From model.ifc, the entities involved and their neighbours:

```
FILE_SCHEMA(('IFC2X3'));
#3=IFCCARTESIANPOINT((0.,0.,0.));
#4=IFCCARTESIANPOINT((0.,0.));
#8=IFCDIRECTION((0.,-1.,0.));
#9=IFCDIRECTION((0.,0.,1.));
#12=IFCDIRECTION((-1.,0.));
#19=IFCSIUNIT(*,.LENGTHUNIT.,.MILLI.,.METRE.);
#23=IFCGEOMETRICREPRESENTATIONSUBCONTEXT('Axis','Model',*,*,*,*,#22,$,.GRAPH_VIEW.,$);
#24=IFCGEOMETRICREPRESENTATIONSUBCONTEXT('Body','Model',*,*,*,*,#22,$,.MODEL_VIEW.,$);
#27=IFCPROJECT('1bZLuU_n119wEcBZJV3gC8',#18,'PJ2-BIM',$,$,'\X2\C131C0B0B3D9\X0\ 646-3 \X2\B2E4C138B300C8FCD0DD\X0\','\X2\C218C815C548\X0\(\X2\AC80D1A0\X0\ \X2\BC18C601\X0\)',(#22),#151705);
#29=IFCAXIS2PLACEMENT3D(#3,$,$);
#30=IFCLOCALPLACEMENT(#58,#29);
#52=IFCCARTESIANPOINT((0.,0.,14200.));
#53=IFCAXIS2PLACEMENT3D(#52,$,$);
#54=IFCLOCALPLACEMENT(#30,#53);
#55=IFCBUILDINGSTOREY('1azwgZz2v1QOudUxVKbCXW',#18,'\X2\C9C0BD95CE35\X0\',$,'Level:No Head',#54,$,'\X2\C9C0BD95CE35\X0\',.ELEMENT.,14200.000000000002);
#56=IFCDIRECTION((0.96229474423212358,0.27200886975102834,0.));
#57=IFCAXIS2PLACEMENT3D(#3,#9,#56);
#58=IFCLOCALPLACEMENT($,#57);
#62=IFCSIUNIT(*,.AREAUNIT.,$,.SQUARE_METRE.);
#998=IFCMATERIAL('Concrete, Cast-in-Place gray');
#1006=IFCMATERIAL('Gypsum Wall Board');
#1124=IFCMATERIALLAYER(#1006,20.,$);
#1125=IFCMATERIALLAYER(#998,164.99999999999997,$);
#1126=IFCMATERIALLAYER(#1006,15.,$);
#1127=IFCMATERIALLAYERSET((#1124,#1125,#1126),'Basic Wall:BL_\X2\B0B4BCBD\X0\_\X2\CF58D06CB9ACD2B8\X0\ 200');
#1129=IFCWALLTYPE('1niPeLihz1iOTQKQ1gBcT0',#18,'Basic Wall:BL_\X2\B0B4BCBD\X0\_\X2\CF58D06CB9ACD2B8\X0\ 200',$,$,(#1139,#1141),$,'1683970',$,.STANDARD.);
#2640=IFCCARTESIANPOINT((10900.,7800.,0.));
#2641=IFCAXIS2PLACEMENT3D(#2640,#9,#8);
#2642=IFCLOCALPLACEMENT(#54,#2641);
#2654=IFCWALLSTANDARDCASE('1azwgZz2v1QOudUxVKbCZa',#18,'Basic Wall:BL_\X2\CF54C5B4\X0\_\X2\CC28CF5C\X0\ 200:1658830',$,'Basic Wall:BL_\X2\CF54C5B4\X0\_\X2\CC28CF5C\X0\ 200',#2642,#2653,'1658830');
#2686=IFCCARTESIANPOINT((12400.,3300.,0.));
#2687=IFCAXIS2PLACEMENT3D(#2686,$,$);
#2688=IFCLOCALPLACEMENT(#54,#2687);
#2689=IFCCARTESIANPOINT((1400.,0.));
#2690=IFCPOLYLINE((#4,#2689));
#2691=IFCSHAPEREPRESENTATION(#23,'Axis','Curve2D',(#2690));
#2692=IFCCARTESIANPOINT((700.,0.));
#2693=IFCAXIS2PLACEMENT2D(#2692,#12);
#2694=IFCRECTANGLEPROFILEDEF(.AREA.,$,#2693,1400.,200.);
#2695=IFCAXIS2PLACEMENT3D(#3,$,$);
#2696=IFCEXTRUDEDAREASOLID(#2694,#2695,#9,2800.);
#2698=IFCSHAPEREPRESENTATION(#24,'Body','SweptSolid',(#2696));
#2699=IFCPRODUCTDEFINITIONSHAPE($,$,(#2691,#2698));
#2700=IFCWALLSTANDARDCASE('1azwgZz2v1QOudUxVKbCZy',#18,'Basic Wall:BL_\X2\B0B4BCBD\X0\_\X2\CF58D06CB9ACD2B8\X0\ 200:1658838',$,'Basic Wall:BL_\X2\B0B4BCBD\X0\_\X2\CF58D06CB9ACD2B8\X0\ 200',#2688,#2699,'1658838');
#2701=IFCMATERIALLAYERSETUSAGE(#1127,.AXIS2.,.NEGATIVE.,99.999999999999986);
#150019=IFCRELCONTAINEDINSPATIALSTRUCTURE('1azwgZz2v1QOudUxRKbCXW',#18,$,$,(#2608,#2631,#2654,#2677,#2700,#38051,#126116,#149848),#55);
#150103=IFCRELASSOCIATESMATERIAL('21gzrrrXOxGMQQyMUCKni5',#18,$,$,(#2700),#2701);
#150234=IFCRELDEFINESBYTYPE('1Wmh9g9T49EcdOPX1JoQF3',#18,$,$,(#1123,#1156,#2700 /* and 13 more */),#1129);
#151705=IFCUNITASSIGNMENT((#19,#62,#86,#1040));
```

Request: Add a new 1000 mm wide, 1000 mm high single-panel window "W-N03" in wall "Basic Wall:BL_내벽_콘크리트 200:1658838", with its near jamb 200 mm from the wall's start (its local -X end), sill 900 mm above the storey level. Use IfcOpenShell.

```python
import numpy as np
import ifcopenshell
import ifcopenshell.api.feature
import ifcopenshell.api.geometry
import ifcopenshell.api.root
import ifcopenshell.api.spatial
import ifcopenshell.api.type
import ifcopenshell.geom
import ifcopenshell.util.element
import ifcopenshell.util.placement
import ifcopenshell.util.representation
import ifcopenshell.util.shape
import ifcopenshell.util.unit

model = ifcopenshell.open("model.ifc")
unit_scale = ifcopenshell.util.unit.calculate_unit_scale(model)
settings = ifcopenshell.geom.settings()


def volume(element):
    """Net volume in cubic metres, openings subtracted."""
    shape = ifcopenshell.geom.create_shape(settings, element)
    return ifcopenshell.util.shape.get_volume(shape.geometry)


wall = model.by_guid("1azwgZz2v1QOudUxVKbCZy")
storey = ifcopenshell.util.element.get_container(wall, ifc_class="IfcBuildingStorey")
context = ifcopenshell.util.representation.get_context(model, "Model", "Body", "MODEL_VIEW")
before = volume(wall)

width, height, from_end, sill = 1, 1, 0.2, 0.9  # metres

# The wall runs along its own X axis, and the end named is its -X end.
wall_shape = ifcopenshell.geom.create_shape(settings, wall)
x, y, z = ifcopenshell.util.shape.get_vertices(wall_shape.geometry).T
start = x.min() + from_end
face, thickness = float(y.min()), float(y.max() - y.min())
wall_matrix = ifcopenshell.util.placement.get_local_placement(wall.ObjectPlacement)
level = ifcopenshell.util.placement.get_local_placement(storey.ObjectPlacement)[2, 3]


def in_wall(x, y):
    """Placement at x, y metres in the wall's axes, at sill height."""
    matrix = wall_matrix.copy()
    matrix[:, 3] = wall_matrix @ np.array([x / unit_scale, y / unit_scale, 0.0, 1.0])
    matrix[2, 3] = level + sill / unit_scale
    return matrix


# Opening: a box that overshoots both wall faces by 50 mm.
opening = ifcopenshell.api.root.create_entity(model, ifc_class="IfcOpeningElement")
box = ifcopenshell.api.geometry.add_wall_representation(
    model, context=context, length=width, height=height, thickness=thickness + 0.1
)
ifcopenshell.api.geometry.assign_representation(model, product=opening, representation=box)
ifcopenshell.api.geometry.edit_object_placement(model, product=opening, matrix=in_wall(start, face - 0.05), is_si=False)
ifcopenshell.api.feature.add_feature(model, feature=opening, element=wall)

window = ifcopenshell.api.root.create_entity(model, ifc_class="IfcWindow", name="W-N03")
window.OverallWidth, window.OverallHeight = width / unit_scale, height / unit_scale
body = ifcopenshell.api.geometry.add_window_representation(
    model,
    context=context,
    overall_width=window.OverallWidth,
    overall_height=window.OverallHeight,
    partition_type="SINGLE_PANEL",
)
ifcopenshell.api.geometry.assign_representation(model, product=window, representation=body)
ifcopenshell.api.spatial.assign_container(model, products=[window], relating_structure=storey)
fills = ifcopenshell.api.feature.add_filling(model, opening=opening, element=window)
fills.OwnerHistory = window.OwnerHistory  # required in IFC2X3

# IFC2X3 keeps the operation on the window style.
style = ifcopenshell.api.root.create_entity(model, ifc_class="IfcWindowStyle", name="W-N03")
style.OperationType, style.ConstructionType = "SINGLE_PANEL", "NOTDEFINED"
style.ParameterTakesPrecedence = style.Sizeable = False
ifcopenshell.api.type.assign_type(model, related_objects=[window], relating_type=style)

# Centre the window in the wall's thickness.
ifcopenshell.api.geometry.edit_object_placement(model, product=window, matrix=in_wall(start, face), is_si=False)
window_shape = ifcopenshell.geom.create_shape(settings, window)
depth = ifcopenshell.util.shape.get_vertices(window_shape.geometry)[:, 1]
offset = face + thickness / 2 - (depth.min() + depth.max()) / 2
ifcopenshell.api.geometry.edit_object_placement(model, product=window, matrix=in_wall(start, offset), is_si=False)

after = volume(wall)

print(f"wall volume {before:.3f} -> {after:.3f} m3")

model.write("model-out.ifc")
```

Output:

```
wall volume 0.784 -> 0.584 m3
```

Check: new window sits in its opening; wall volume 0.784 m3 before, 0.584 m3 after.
